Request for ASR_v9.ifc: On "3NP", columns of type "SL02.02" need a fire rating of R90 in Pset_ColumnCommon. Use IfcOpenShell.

First a look at what the model holds.

```python
import ifcopenshell
import ifcopenshell.util.element

model = ifcopenshell.open("ASR_v9.ifc")
print(model.schema)
storey = next(s for s in model.by_type("IfcBuildingStorey") if s.Name == "3NP")
columns = [e for e in ifcopenshell.util.element.get_decomposition(storey) if e.is_a("IfcColumn")]
seen = {}
for e in columns:
    element_type = ifcopenshell.util.element.get_type(e)
    key = (element_type.Name if element_type != e and element_type else None, ifcopenshell.util.element.get_pset(e, "Pset_ColumnCommon", "FireRating"))
    seen[key] = seen.get(key, 0) + 1
for (name, value), count in sorted(seen.items(), key=str):
    print(count, "x", name, "|", value)
```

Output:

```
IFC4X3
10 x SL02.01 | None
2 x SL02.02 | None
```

```python
import ifcopenshell
import ifcopenshell.api.pset
import ifcopenshell.util.element

model = ifcopenshell.open("ASR_v9.ifc")

storey = next(s for s in model.by_type("IfcBuildingStorey") if s.Name == "3NP")
columns = [e for e in ifcopenshell.util.element.get_decomposition(storey) if e.is_a("IfcColumn")]

count = 0
for e in columns:
    element_type = ifcopenshell.util.element.get_type(e)
    if element_type in (None, e) or element_type.Name != "SL02.02":
        continue
    # add_pset returns the element's existing set when there is one.
    pset = ifcopenshell.api.pset.add_pset(model, product=e, name="Pset_ColumnCommon")
    ifcopenshell.api.pset.edit_pset(model, pset=pset, properties={"FireRating": "R90"})
    count += 1

print(count, "columns updated")

model.write("ASR_v9_updated.ifc")
```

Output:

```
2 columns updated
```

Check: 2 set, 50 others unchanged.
